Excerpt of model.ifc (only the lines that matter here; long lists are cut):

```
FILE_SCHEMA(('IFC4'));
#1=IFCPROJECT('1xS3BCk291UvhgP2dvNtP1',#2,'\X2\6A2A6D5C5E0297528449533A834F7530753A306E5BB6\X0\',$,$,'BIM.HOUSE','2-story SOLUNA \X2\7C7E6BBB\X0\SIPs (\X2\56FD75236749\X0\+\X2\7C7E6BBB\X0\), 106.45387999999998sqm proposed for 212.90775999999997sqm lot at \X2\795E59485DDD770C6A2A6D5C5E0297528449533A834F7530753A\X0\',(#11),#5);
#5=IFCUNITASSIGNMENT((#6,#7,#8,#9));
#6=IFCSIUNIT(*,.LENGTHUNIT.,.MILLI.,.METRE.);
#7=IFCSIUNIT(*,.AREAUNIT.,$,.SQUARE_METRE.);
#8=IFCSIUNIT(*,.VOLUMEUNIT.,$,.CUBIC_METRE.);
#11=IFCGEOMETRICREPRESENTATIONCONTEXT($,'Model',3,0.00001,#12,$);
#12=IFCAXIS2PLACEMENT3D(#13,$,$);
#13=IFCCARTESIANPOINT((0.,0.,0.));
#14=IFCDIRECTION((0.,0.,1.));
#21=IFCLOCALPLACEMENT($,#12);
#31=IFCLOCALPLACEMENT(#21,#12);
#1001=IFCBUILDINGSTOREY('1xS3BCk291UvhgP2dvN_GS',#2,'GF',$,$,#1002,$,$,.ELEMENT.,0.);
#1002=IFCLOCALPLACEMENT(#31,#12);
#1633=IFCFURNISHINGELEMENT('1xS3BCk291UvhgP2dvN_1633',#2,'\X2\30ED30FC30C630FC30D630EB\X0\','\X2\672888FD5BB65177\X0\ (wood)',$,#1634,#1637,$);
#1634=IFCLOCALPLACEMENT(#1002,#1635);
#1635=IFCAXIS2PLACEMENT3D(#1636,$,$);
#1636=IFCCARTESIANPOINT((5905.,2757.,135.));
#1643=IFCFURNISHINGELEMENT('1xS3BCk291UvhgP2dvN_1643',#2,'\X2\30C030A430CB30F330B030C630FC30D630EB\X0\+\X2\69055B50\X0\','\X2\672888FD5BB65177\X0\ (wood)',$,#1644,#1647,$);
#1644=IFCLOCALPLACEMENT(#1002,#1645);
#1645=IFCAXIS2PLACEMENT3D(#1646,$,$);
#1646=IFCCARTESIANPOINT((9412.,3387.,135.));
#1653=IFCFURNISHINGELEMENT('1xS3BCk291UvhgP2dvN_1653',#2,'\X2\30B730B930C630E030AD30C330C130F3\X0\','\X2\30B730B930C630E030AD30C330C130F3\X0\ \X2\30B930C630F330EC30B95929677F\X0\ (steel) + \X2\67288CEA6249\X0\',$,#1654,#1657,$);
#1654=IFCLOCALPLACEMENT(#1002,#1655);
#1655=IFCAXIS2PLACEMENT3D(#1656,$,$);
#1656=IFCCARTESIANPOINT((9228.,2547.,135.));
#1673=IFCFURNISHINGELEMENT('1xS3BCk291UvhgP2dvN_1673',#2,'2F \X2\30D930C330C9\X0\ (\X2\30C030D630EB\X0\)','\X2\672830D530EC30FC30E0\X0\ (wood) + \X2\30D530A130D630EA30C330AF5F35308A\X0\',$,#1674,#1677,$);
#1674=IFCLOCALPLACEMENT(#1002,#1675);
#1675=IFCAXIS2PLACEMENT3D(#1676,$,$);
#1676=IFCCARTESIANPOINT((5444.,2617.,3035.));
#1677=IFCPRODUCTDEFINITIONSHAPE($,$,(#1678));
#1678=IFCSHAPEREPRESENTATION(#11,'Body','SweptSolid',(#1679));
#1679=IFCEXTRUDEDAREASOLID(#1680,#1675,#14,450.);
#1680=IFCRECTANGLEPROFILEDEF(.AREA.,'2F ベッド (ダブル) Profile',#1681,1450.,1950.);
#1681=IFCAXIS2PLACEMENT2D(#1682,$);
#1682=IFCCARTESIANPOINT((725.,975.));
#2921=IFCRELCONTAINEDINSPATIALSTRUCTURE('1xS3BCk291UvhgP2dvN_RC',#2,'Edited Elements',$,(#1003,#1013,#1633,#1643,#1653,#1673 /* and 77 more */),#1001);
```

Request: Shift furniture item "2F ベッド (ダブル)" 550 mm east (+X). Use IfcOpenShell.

```python
import ifcopenshell
import ifcopenshell.api.geometry
import ifcopenshell.util.placement
import ifcopenshell.util.unit

model = ifcopenshell.open("model.ifc")
unit_scale = ifcopenshell.util.unit.calculate_unit_scale(model)

item = model.by_id(1673)
matrix = ifcopenshell.util.placement.get_local_placement(item.ObjectPlacement)
matrix[0, 3] += 0.55 / unit_scale
ifcopenshell.api.geometry.edit_object_placement(model, product=item, matrix=matrix, is_si=False)

print(ifcopenshell.util.placement.get_local_placement(item.ObjectPlacement).round(3) + 0.0)

model.write("model_edited.ifc")
```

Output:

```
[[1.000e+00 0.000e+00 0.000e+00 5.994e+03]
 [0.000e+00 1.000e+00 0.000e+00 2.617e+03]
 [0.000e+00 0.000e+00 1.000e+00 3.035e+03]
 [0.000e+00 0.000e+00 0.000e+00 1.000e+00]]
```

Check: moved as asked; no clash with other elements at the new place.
